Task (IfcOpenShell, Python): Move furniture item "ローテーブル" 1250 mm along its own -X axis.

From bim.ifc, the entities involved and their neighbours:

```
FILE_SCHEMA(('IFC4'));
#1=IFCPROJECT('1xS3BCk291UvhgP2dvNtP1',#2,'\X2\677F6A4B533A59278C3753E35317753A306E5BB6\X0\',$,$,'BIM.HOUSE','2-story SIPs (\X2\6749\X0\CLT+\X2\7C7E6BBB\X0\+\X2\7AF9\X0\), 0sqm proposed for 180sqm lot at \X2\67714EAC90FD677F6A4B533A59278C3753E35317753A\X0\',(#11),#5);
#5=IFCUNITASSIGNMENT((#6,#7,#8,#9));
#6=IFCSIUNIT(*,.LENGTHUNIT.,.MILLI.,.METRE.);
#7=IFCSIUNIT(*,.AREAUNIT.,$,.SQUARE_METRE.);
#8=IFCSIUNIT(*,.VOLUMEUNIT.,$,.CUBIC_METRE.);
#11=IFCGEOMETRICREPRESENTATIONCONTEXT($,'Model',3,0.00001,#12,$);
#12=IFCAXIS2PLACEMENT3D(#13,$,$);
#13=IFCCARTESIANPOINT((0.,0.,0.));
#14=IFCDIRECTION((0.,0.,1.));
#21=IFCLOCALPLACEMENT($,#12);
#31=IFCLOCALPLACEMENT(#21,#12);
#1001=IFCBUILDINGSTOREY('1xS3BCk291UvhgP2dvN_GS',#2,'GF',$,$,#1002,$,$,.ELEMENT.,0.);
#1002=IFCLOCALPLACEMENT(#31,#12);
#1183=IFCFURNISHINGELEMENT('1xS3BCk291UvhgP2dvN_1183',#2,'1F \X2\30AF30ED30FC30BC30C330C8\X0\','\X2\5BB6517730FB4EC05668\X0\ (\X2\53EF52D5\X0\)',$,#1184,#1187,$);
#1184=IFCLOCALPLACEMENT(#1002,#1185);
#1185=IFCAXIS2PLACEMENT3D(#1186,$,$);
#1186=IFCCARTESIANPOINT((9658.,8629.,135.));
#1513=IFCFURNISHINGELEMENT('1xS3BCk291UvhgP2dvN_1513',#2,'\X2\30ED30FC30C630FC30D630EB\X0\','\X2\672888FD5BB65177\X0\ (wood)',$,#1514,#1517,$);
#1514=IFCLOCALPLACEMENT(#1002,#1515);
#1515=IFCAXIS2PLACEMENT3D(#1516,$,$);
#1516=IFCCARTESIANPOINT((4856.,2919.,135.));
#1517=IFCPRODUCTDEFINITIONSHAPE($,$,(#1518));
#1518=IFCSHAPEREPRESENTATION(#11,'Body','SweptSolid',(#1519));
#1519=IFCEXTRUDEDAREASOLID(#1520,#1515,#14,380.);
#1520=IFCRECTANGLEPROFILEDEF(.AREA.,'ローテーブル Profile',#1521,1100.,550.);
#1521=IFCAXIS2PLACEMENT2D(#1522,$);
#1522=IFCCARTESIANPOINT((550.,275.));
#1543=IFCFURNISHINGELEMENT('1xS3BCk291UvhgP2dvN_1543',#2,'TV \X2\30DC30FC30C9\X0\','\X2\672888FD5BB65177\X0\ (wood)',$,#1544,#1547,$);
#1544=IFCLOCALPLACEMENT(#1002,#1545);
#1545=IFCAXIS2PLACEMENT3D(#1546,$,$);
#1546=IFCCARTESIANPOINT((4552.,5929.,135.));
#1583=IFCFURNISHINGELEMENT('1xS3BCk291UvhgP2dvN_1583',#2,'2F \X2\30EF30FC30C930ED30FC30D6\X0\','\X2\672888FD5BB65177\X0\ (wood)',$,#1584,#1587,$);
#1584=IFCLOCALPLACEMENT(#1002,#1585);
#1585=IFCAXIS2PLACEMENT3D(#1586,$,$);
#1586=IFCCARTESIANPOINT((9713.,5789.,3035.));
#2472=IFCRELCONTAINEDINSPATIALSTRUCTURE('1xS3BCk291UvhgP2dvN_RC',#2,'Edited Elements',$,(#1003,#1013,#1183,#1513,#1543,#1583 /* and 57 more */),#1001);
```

```python
import ifcopenshell
import ifcopenshell.api.geometry
import ifcopenshell.util.placement
import ifcopenshell.util.unit

model = ifcopenshell.open("bim.ifc")
unit_scale = ifcopenshell.util.unit.calculate_unit_scale(model)

item = model.by_guid("1xS3BCk291UvhgP2dvN_1513")
matrix = ifcopenshell.util.placement.get_local_placement(item.ObjectPlacement)
matrix[:3, 3] -= matrix[:3, 0] * 1.25 / unit_scale
ifcopenshell.api.geometry.edit_object_placement(model, product=item, matrix=matrix, is_si=False)

print(ifcopenshell.util.placement.get_local_placement(item.ObjectPlacement).round(3) + 0.0)

model.write("bim_edited.ifc")
```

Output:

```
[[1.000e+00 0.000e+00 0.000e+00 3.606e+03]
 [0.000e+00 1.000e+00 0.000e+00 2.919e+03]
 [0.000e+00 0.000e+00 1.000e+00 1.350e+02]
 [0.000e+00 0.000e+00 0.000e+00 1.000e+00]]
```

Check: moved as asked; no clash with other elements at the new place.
